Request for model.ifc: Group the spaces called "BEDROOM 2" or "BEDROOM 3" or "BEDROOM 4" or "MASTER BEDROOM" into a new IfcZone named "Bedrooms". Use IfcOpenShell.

First a look at what the model holds.

```python
import ifcopenshell

model = ifcopenshell.open("model.ifc")
print(model.schema)
seen = {}
for space in model.by_type("IfcSpace"):
    seen[space.LongName] = seen.get(space.LongName, 0) + 1
for name, count in sorted(seen.items(), key=str):
    print(count, "x", name)
print("zones:", [z.Name for z in model.by_type("IfcZone")][:20])
```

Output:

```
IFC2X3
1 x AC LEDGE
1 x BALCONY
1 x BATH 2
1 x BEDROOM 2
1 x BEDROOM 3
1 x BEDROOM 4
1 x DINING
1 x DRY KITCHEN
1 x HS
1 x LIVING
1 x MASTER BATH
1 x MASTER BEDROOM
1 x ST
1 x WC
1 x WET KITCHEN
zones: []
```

```python
import ifcopenshell
import ifcopenshell.api.group
import ifcopenshell.api.root

model = ifcopenshell.open("model.ifc")

names = {"BEDROOM 2", "BEDROOM 3", "BEDROOM 4", "MASTER BEDROOM"}
spaces = [s for s in model.by_type("IfcSpace") if s.LongName in names]

zone = ifcopenshell.api.root.create_entity(model, ifc_class="IfcZone", name="Bedrooms")
ifcopenshell.api.group.assign_group(model, products=spaces, group=zone)
print(len(spaces), "spaces in", zone.Name)

model.write("model_edited.ifc")
```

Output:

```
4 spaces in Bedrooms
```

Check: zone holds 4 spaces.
